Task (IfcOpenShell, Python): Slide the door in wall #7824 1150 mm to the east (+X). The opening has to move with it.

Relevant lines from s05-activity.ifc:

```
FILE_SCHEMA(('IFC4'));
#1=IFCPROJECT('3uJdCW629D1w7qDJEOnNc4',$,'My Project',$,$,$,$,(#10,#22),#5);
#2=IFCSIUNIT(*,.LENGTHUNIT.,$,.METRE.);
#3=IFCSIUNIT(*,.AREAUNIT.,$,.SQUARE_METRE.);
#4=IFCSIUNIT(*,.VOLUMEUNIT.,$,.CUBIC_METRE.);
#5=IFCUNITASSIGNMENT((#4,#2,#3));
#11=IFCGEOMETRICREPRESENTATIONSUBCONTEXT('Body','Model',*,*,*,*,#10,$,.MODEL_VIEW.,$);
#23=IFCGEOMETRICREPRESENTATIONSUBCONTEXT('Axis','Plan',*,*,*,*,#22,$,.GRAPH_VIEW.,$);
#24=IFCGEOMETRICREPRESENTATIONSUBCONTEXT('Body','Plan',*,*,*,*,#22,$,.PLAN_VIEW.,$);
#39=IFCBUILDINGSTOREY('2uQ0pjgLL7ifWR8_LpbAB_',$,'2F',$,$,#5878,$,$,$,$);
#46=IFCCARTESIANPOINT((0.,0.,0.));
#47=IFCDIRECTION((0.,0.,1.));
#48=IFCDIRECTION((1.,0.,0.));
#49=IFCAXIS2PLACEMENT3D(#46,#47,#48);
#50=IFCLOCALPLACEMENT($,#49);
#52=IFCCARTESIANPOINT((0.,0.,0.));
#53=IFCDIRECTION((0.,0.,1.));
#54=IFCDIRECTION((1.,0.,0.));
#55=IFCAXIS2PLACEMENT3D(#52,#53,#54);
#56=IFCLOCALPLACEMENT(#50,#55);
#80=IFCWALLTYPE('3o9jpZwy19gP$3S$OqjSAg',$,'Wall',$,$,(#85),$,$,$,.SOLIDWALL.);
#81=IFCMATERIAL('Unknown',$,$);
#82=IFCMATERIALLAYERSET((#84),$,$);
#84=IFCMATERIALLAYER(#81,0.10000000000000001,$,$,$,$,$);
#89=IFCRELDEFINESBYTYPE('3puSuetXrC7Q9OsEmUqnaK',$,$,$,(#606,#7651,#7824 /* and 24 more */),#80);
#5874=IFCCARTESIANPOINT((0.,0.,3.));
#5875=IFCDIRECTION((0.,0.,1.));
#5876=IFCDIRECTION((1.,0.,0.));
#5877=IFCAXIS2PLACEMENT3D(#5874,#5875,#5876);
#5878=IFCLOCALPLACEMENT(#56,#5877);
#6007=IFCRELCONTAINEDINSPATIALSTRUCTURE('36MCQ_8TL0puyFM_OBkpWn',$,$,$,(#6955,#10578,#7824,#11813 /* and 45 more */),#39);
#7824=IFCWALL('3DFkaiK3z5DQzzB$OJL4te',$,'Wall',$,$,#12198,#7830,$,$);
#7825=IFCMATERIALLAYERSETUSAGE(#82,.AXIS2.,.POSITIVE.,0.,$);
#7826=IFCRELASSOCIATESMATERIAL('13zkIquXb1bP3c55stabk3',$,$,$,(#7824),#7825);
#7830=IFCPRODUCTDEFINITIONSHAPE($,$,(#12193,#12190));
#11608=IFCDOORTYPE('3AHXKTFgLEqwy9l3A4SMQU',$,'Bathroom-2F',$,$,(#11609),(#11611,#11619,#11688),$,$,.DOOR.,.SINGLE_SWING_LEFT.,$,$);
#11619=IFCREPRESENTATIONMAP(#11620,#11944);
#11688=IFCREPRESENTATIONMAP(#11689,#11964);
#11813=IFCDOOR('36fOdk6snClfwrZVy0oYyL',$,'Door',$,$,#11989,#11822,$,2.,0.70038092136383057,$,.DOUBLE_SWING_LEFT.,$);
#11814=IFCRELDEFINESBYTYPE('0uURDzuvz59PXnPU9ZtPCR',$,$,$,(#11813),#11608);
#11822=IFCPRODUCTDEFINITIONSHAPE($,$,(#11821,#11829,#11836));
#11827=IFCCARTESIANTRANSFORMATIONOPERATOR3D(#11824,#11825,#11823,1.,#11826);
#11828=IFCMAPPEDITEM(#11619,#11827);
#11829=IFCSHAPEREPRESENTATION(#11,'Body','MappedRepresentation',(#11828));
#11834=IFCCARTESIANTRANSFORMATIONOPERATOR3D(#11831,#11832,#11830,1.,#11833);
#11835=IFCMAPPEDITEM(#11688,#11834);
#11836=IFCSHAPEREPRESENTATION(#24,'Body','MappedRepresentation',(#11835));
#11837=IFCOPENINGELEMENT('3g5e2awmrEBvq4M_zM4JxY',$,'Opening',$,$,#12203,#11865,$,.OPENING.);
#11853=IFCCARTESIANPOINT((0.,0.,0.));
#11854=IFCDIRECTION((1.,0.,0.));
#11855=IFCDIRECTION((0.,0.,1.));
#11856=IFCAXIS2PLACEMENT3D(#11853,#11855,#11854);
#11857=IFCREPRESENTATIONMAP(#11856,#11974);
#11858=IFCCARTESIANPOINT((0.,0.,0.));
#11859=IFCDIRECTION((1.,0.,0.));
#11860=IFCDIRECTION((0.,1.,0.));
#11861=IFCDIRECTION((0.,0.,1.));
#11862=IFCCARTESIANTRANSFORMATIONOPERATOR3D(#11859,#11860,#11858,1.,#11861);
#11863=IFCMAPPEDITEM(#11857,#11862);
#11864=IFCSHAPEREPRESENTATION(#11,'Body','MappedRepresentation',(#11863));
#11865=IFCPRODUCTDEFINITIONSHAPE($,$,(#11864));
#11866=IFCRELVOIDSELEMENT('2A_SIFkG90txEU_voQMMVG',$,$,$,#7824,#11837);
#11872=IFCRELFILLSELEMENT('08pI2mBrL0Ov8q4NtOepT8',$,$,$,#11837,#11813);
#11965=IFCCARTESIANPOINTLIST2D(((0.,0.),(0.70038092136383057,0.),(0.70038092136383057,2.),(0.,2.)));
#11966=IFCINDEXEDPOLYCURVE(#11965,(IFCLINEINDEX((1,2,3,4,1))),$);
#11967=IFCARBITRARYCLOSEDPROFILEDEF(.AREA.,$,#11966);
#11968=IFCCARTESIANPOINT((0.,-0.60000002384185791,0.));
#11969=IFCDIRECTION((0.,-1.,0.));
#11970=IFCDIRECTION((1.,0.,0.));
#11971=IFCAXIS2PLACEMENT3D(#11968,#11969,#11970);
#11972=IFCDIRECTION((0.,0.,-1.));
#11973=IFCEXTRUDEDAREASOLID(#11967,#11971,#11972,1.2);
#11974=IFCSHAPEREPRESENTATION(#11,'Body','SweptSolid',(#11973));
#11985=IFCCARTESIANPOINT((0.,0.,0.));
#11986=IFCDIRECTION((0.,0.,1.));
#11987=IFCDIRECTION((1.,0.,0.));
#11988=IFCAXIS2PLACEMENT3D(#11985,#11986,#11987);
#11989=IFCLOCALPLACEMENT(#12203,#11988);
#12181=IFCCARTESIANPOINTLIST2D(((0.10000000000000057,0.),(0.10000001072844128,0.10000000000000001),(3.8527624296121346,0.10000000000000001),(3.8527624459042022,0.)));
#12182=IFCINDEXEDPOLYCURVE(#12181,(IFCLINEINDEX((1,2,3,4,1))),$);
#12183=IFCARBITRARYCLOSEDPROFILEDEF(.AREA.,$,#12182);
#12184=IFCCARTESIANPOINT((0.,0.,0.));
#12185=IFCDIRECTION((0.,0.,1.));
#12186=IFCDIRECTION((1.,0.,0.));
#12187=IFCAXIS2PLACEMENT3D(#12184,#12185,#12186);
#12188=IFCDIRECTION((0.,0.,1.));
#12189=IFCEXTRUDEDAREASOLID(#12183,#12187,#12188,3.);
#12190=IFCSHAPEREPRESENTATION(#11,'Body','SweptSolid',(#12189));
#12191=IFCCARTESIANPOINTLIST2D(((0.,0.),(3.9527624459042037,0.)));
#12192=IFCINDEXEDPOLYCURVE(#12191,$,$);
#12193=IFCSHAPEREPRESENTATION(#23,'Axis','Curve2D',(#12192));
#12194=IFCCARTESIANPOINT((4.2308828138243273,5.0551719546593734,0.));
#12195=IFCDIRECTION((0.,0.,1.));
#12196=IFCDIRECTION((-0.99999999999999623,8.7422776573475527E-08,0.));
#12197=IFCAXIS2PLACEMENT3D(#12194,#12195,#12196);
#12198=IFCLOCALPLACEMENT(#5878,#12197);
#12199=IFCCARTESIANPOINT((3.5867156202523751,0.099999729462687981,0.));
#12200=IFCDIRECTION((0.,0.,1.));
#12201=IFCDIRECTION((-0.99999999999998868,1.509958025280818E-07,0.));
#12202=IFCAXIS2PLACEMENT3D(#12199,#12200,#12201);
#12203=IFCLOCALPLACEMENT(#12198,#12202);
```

```python
import ifcopenshell
import ifcopenshell.api.geometry
import ifcopenshell.util.placement
import ifcopenshell.util.unit

model = ifcopenshell.open("s05-activity.ifc")
unit_scale = ifcopenshell.util.unit.calculate_unit_scale(model)

door = model.by_guid("36fOdk6snClfwrZVy0oYyL")
opening = door.FillsVoids[0].RelatingOpeningElement
wall = opening.VoidsElements[0].RelatingBuildingElement

wall_matrix = ifcopenshell.util.placement.get_local_placement(wall.ObjectPlacement)
shift = wall_matrix[:3, 0] * -1.15 / unit_scale
before = ifcopenshell.util.placement.get_local_placement(door.ObjectPlacement)[:3, 3].copy()

# The door is placed relative to its opening, so it follows when the opening moves.
matrix = ifcopenshell.util.placement.get_local_placement(opening.ObjectPlacement)
matrix[:3, 3] += shift
ifcopenshell.api.geometry.edit_object_placement(
    model, product=opening, matrix=matrix, is_si=False, should_transform_children=True
)

after = ifcopenshell.util.placement.get_local_placement(door.ObjectPlacement)[:3, 3]
print("door moved by", (after - before).round(3) + 0.0)

model.write("s05-activity_v2.ifc")
```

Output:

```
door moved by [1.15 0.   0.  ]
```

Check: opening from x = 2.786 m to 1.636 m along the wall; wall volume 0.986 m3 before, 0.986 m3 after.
